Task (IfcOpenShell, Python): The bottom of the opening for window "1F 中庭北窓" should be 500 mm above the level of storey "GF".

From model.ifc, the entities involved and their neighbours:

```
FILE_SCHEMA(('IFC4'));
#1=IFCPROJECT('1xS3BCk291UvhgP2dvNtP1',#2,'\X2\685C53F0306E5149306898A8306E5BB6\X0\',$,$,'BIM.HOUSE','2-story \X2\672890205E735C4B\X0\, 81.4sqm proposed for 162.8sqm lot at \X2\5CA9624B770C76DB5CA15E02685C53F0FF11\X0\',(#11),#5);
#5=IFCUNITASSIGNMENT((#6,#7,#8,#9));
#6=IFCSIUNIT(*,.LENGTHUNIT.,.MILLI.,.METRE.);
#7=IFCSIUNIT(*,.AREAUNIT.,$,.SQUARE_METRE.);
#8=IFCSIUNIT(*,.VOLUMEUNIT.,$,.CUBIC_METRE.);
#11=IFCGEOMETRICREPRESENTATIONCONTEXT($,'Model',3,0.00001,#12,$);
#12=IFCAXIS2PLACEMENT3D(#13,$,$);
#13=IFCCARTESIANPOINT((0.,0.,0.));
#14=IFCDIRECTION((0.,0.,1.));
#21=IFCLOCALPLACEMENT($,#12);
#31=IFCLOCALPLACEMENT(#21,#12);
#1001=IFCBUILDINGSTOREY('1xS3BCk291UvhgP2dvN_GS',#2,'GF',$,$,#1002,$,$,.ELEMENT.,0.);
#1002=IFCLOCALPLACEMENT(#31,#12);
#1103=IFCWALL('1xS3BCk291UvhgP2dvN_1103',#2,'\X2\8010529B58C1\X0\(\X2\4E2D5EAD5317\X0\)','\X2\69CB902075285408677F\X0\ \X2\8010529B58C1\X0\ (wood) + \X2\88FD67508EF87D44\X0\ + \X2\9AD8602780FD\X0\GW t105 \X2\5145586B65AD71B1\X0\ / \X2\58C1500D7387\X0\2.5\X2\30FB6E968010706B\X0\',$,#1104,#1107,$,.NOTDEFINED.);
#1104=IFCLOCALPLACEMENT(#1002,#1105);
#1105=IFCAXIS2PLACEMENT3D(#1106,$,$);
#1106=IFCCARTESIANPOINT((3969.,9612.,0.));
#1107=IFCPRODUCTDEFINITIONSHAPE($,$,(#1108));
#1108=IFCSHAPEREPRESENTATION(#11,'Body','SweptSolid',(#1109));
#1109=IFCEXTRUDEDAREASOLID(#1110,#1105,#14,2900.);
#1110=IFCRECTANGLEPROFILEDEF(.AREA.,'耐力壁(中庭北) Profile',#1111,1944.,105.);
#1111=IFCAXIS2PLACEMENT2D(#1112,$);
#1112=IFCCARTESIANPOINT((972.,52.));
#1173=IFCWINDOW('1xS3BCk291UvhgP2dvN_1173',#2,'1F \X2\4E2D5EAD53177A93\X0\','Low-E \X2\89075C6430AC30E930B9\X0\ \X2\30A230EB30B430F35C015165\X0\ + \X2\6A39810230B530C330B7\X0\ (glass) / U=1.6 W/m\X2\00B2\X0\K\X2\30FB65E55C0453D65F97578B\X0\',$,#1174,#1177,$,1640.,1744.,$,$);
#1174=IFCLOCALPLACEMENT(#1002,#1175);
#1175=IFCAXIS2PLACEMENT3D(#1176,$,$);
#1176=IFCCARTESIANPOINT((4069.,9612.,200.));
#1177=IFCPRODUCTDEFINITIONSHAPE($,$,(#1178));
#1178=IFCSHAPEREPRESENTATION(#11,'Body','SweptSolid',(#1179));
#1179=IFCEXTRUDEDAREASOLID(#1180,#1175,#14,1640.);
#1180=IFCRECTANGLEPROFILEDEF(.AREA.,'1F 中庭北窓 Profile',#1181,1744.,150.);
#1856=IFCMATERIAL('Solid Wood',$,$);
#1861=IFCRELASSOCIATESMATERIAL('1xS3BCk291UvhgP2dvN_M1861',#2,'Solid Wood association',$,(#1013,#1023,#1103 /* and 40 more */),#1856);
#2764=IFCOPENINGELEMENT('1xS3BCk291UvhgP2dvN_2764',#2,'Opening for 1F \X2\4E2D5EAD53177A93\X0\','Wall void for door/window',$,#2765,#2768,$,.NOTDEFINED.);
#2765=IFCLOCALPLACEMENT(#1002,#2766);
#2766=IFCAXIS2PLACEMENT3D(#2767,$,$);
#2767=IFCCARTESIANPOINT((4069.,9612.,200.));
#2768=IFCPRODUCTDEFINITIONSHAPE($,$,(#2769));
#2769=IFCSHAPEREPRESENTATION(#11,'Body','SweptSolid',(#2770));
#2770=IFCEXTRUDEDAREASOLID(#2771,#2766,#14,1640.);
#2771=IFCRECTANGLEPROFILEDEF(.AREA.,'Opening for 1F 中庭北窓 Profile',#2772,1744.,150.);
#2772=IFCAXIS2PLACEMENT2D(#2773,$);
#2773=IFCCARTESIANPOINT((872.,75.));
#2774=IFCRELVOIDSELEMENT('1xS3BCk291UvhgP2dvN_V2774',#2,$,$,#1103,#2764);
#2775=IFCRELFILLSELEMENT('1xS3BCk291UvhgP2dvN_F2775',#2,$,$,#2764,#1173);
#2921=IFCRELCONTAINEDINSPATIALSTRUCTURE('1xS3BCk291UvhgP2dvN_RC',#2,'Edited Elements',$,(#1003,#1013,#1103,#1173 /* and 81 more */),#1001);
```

```python
import numpy as np
import ifcopenshell
import ifcopenshell.api.geometry
import ifcopenshell.geom
import ifcopenshell.util.element
import ifcopenshell.util.placement
import ifcopenshell.util.shape
import ifcopenshell.util.unit

model = ifcopenshell.open("model.ifc")
unit_scale = ifcopenshell.util.unit.calculate_unit_scale(model)

window = model.by_guid("1xS3BCk291UvhgP2dvN_1173")
opening = window.FillsVoids[0].RelatingOpeningElement
storey = ifcopenshell.util.element.get_container(window, ifc_class="IfcBuildingStorey")
level = ifcopenshell.util.placement.get_local_placement(storey.ObjectPlacement)[2, 3]

# The opening's origin need not be at the sill, so measure its lowest point.
shape = ifcopenshell.geom.create_shape(ifcopenshell.geom.settings(), opening)
bottom = ifcopenshell.util.shape.get_shape_bottom_elevation(shape, shape.geometry) / unit_scale
dz = level + 0.5 / unit_scale - bottom

shift = np.array([0.0, 0.0, dz])
# The window is not placed relative to its opening, so move both.
for product in (opening, window):
    matrix = ifcopenshell.util.placement.get_local_placement(product.ObjectPlacement)
    matrix[:3, 3] += shift
    ifcopenshell.api.geometry.edit_object_placement(model, product=product, matrix=matrix, is_si=False)

print(f"moved by {dz * unit_scale:+.3f} m")

model.write("model_edited.ifc")
```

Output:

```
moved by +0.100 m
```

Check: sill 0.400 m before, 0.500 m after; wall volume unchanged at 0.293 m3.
